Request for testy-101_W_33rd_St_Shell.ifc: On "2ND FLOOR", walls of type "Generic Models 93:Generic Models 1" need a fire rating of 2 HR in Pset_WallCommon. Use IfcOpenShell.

First a look at what the model holds.

```python
import ifcopenshell
import ifcopenshell.util.element

model = ifcopenshell.open("testy-101_W_33rd_St_Shell.ifc")
print(model.schema)
storey = next(s for s in model.by_type("IfcBuildingStorey") if s.Name == "2ND FLOOR")
walls = [e for e in ifcopenshell.util.element.get_decomposition(storey) if e.is_a("IfcWall")]
seen = {}
for e in walls:
    element_type = ifcopenshell.util.element.get_type(e)
    key = (element_type.Name if element_type != e and element_type else None, ifcopenshell.util.element.get_pset(e, "Pset_WallCommon", "FireRating"))
    seen[key] = seen.get(key, 0) + 1
for (name, value), count in sorted(seen.items(), key=str):
    print(count, "x", name, "|", value)
```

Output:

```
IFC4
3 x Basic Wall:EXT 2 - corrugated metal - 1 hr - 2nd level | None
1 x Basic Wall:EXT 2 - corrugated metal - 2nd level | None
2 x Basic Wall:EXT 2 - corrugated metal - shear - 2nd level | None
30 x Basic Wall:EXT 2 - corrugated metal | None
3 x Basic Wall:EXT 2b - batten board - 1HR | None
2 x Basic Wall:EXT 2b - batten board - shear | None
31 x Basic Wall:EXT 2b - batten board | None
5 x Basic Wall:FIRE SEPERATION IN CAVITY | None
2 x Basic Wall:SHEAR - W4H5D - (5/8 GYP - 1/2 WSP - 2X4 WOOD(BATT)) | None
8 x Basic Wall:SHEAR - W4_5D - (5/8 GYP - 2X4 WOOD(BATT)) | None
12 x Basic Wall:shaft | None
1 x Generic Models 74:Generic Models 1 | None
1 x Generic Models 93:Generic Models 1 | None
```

```python
import ifcopenshell
import ifcopenshell.api.pset
import ifcopenshell.util.element

model = ifcopenshell.open("testy-101_W_33rd_St_Shell.ifc")

storey = next(s for s in model.by_type("IfcBuildingStorey") if s.Name == "2ND FLOOR")
walls = [e for e in ifcopenshell.util.element.get_decomposition(storey) if e.is_a("IfcWall")]

count = 0
for e in walls:
    element_type = ifcopenshell.util.element.get_type(e)
    if element_type in (None, e) or element_type.Name != "Generic Models 93:Generic Models 1":
        continue
    # add_pset returns the element's existing set when there is one.
    pset = ifcopenshell.api.pset.add_pset(model, product=e, name="Pset_WallCommon")
    ifcopenshell.api.pset.edit_pset(model, pset=pset, properties={"FireRating": "2 HR"})
    count += 1

print(count, "walls updated")

model.write("testy-101_W_33rd_St_Shell-out.ifc")
```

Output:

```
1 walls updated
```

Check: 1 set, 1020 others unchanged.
